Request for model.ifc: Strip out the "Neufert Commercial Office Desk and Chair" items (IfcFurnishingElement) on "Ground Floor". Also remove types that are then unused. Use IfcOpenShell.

First a look at what the model holds.

```python
import ifcopenshell
import ifcopenshell.util.element

model = ifcopenshell.open("model.ifc")
print(model.schema)
storey = next(s for s in model.by_type("IfcBuildingStorey") if s.Name == "Ground Floor")
furniture = [e for e in ifcopenshell.util.element.get_decomposition(storey) if e.is_a("IfcFurnishingElement")]
seen = {}
for e in furniture:
    element_type = ifcopenshell.util.element.get_type(e)
    name = element_type.Name if element_type not in (None, e) else None
    seen[name] = seen.get(name, 0) + 1
for name, count in sorted(seen.items(), key=str):
    print(count, "x", name)
```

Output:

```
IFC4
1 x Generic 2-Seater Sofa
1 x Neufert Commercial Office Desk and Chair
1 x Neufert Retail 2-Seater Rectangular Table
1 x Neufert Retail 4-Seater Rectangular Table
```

```python
import ifcopenshell
import ifcopenshell.api.root
import ifcopenshell.util.element

model = ifcopenshell.open("model.ifc")

storey = next(s for s in model.by_type("IfcBuildingStorey") if s.Name == "Ground Floor")
furniture = [e for e in ifcopenshell.util.element.get_decomposition(storey) if e.is_a("IfcFurnishingElement")]
targets = [e for e in furniture if (t := ifcopenshell.util.element.get_type(e)) not in (None, e) and t.Name == "Neufert Commercial Office Desk and Chair"]
types = {ifcopenshell.util.element.get_type(e) for e in targets} - {None, *targets}

for e in targets:
    ifcopenshell.api.root.remove_product(model, product=e)
print(len(targets), "removed")

unused = [t for t in types if not ifcopenshell.util.element.get_types(t)]
for t in unused:
    ifcopenshell.api.root.remove_product(model, product=t)
print(len(unused), "unused types removed")

model.write("model_updated.ifc")
```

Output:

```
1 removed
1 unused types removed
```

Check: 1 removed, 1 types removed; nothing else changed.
